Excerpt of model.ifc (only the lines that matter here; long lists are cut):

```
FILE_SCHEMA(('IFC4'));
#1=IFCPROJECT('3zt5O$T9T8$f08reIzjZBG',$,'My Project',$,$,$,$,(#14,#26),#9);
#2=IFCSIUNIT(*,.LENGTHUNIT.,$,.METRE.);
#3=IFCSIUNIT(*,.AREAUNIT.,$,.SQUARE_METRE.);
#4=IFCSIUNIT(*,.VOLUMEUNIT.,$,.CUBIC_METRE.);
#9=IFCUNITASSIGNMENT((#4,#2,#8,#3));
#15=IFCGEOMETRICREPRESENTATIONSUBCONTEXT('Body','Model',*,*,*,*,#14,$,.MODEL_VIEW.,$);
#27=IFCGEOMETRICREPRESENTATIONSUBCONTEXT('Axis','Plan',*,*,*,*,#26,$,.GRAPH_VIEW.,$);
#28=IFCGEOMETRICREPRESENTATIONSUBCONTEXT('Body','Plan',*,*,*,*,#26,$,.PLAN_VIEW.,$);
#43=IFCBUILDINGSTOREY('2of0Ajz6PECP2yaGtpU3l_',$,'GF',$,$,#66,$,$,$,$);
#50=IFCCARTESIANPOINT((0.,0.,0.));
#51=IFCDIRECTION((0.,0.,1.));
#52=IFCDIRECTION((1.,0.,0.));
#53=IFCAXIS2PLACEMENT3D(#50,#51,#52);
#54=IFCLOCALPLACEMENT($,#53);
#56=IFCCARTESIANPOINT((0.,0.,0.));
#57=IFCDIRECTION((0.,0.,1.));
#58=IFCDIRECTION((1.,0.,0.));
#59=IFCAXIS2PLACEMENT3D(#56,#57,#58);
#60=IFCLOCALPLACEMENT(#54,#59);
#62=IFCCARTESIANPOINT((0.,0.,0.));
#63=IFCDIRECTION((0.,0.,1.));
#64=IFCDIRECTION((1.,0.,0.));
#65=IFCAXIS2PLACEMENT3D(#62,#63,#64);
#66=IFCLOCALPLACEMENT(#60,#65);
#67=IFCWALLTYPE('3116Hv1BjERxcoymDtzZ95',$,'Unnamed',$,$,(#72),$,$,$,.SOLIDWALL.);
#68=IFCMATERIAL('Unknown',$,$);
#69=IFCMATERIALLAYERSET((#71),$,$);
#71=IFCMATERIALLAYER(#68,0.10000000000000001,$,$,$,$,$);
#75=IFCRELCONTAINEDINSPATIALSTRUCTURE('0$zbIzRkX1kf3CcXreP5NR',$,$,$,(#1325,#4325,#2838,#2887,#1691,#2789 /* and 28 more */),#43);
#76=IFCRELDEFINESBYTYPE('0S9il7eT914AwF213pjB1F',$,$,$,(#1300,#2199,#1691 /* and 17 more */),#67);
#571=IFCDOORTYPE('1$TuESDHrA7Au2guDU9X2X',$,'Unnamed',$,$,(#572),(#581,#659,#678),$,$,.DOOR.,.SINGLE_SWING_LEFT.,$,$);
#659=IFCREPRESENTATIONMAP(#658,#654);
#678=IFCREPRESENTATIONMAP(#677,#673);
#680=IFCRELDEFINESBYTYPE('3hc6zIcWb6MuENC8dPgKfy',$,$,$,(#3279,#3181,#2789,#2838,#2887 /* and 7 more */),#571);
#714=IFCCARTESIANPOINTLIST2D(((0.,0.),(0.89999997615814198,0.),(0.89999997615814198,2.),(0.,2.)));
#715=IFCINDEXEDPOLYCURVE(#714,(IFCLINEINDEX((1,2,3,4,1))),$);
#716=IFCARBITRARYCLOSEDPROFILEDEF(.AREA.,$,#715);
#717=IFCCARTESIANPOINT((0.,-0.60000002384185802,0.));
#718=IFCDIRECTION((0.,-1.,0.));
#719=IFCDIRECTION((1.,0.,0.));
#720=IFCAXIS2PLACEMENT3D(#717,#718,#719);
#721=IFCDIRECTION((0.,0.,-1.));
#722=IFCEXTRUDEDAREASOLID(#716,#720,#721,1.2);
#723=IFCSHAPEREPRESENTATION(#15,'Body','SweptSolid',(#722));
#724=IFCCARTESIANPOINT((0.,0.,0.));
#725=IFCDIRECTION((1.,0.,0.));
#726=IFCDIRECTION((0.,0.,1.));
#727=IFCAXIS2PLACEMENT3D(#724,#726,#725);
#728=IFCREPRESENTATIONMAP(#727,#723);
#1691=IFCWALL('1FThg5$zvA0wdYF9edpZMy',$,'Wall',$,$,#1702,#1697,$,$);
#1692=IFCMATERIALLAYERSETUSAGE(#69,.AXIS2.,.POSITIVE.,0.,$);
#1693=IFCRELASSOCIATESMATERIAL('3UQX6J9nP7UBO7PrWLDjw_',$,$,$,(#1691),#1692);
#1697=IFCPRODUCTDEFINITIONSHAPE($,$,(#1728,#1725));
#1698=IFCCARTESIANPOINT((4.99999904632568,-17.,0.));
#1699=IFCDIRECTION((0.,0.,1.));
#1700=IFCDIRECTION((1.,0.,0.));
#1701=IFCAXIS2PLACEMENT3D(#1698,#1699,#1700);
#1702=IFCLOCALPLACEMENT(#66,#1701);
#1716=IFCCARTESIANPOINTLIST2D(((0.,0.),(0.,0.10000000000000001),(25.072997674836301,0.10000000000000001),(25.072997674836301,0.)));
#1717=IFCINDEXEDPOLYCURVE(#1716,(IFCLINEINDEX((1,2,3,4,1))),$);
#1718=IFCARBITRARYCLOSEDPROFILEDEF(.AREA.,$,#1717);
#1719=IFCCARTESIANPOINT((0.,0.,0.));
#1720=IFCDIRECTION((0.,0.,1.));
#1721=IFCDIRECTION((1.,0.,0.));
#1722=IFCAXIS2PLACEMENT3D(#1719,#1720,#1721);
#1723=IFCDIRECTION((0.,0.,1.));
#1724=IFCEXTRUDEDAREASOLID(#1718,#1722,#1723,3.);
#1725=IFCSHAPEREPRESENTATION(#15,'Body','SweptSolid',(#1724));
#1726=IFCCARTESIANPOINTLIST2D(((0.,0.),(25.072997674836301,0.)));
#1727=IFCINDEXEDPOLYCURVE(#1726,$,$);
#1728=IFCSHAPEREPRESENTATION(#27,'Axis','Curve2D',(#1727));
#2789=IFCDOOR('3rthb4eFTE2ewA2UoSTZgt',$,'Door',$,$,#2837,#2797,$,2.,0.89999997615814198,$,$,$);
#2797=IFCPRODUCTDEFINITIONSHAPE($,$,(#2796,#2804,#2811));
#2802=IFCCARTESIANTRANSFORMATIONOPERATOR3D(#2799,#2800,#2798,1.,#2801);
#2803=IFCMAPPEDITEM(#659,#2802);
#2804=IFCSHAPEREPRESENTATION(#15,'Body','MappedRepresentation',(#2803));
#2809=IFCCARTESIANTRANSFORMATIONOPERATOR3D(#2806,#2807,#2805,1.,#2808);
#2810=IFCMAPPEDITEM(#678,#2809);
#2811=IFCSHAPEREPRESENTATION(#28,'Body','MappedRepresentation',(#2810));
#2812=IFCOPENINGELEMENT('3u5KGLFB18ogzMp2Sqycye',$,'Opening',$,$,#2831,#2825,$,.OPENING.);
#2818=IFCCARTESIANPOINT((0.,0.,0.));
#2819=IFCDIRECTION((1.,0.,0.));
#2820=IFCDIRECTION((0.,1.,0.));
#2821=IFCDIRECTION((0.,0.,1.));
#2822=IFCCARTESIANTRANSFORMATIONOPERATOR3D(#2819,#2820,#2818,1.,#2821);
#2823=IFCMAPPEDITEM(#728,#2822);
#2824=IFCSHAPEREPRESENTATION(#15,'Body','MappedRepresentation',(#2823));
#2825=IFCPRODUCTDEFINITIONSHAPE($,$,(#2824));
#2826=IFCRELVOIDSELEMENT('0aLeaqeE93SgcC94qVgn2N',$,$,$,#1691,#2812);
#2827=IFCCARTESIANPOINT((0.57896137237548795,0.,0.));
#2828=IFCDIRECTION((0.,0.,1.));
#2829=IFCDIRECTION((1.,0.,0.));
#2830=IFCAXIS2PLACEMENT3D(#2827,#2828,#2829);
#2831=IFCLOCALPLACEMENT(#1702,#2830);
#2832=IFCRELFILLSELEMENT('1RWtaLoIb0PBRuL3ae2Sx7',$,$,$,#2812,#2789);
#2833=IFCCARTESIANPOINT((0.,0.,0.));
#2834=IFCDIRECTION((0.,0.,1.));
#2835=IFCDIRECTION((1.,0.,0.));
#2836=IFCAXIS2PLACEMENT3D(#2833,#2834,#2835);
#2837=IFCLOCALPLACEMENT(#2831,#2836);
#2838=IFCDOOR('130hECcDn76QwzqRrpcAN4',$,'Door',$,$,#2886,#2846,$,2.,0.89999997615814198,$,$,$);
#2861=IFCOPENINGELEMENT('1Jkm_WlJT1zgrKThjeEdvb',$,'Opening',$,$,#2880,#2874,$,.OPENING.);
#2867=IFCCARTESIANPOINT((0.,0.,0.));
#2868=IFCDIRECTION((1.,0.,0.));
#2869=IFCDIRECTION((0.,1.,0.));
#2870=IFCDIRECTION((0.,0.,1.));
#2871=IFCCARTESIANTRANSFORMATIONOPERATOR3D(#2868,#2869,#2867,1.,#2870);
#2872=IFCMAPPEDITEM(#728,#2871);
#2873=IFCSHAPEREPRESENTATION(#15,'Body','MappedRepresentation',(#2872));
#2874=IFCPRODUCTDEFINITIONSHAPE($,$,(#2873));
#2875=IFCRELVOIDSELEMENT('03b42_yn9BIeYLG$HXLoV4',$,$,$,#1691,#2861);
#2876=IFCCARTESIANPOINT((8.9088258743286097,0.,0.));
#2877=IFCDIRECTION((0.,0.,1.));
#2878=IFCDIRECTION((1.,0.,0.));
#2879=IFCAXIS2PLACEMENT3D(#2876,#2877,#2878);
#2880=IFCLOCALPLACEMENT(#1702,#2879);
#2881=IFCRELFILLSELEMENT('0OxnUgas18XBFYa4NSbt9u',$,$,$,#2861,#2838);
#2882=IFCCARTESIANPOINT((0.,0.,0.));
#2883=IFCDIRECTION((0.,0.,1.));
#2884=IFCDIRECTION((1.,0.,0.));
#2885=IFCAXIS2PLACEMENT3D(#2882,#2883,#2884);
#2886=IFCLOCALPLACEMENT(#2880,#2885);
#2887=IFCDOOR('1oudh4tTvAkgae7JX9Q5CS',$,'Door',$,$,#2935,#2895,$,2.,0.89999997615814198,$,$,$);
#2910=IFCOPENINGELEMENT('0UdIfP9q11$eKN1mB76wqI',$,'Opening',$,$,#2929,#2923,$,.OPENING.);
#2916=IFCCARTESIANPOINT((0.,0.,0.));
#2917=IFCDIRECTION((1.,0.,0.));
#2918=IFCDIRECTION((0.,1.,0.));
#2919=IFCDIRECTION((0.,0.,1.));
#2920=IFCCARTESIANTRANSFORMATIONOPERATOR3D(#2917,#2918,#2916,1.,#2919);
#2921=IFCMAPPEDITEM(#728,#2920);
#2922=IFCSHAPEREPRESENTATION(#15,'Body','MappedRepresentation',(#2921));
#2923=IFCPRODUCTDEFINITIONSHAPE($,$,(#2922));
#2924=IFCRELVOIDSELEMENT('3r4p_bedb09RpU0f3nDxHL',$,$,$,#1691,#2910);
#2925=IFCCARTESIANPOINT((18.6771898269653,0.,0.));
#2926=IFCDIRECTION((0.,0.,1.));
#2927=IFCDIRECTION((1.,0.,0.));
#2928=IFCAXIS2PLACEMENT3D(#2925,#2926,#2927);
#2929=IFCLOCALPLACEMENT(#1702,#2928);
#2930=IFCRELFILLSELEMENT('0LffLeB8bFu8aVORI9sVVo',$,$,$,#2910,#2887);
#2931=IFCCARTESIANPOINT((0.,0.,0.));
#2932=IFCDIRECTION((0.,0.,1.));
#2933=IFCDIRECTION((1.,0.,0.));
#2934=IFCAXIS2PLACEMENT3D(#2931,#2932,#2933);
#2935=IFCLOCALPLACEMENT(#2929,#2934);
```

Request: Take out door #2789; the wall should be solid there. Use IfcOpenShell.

```python
import ifcopenshell
import ifcopenshell.api.feature
import ifcopenshell.api.root
import ifcopenshell.geom
import ifcopenshell.util.shape

model = ifcopenshell.open("model.ifc")
settings = ifcopenshell.geom.settings()


def volume(element):
    """Net volume in cubic metres, openings subtracted."""
    shape = ifcopenshell.geom.create_shape(settings, element)
    return ifcopenshell.util.shape.get_volume(shape.geometry)


door = model.by_guid("3rthb4eFTE2ewA2UoSTZgt")
opening = door.FillsVoids[0].RelatingOpeningElement
wall = opening.VoidsElements[0].RelatingBuildingElement
before = volume(wall)

ifcopenshell.api.root.remove_product(model, product=door)
ifcopenshell.api.feature.remove_feature(model, feature=opening)

after = volume(wall)

print(f"wall volume {before:.3f} -> {after:.3f} m3")

model.write("model_v2.ifc")
```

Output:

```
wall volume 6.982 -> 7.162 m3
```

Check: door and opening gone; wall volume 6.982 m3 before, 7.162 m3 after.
